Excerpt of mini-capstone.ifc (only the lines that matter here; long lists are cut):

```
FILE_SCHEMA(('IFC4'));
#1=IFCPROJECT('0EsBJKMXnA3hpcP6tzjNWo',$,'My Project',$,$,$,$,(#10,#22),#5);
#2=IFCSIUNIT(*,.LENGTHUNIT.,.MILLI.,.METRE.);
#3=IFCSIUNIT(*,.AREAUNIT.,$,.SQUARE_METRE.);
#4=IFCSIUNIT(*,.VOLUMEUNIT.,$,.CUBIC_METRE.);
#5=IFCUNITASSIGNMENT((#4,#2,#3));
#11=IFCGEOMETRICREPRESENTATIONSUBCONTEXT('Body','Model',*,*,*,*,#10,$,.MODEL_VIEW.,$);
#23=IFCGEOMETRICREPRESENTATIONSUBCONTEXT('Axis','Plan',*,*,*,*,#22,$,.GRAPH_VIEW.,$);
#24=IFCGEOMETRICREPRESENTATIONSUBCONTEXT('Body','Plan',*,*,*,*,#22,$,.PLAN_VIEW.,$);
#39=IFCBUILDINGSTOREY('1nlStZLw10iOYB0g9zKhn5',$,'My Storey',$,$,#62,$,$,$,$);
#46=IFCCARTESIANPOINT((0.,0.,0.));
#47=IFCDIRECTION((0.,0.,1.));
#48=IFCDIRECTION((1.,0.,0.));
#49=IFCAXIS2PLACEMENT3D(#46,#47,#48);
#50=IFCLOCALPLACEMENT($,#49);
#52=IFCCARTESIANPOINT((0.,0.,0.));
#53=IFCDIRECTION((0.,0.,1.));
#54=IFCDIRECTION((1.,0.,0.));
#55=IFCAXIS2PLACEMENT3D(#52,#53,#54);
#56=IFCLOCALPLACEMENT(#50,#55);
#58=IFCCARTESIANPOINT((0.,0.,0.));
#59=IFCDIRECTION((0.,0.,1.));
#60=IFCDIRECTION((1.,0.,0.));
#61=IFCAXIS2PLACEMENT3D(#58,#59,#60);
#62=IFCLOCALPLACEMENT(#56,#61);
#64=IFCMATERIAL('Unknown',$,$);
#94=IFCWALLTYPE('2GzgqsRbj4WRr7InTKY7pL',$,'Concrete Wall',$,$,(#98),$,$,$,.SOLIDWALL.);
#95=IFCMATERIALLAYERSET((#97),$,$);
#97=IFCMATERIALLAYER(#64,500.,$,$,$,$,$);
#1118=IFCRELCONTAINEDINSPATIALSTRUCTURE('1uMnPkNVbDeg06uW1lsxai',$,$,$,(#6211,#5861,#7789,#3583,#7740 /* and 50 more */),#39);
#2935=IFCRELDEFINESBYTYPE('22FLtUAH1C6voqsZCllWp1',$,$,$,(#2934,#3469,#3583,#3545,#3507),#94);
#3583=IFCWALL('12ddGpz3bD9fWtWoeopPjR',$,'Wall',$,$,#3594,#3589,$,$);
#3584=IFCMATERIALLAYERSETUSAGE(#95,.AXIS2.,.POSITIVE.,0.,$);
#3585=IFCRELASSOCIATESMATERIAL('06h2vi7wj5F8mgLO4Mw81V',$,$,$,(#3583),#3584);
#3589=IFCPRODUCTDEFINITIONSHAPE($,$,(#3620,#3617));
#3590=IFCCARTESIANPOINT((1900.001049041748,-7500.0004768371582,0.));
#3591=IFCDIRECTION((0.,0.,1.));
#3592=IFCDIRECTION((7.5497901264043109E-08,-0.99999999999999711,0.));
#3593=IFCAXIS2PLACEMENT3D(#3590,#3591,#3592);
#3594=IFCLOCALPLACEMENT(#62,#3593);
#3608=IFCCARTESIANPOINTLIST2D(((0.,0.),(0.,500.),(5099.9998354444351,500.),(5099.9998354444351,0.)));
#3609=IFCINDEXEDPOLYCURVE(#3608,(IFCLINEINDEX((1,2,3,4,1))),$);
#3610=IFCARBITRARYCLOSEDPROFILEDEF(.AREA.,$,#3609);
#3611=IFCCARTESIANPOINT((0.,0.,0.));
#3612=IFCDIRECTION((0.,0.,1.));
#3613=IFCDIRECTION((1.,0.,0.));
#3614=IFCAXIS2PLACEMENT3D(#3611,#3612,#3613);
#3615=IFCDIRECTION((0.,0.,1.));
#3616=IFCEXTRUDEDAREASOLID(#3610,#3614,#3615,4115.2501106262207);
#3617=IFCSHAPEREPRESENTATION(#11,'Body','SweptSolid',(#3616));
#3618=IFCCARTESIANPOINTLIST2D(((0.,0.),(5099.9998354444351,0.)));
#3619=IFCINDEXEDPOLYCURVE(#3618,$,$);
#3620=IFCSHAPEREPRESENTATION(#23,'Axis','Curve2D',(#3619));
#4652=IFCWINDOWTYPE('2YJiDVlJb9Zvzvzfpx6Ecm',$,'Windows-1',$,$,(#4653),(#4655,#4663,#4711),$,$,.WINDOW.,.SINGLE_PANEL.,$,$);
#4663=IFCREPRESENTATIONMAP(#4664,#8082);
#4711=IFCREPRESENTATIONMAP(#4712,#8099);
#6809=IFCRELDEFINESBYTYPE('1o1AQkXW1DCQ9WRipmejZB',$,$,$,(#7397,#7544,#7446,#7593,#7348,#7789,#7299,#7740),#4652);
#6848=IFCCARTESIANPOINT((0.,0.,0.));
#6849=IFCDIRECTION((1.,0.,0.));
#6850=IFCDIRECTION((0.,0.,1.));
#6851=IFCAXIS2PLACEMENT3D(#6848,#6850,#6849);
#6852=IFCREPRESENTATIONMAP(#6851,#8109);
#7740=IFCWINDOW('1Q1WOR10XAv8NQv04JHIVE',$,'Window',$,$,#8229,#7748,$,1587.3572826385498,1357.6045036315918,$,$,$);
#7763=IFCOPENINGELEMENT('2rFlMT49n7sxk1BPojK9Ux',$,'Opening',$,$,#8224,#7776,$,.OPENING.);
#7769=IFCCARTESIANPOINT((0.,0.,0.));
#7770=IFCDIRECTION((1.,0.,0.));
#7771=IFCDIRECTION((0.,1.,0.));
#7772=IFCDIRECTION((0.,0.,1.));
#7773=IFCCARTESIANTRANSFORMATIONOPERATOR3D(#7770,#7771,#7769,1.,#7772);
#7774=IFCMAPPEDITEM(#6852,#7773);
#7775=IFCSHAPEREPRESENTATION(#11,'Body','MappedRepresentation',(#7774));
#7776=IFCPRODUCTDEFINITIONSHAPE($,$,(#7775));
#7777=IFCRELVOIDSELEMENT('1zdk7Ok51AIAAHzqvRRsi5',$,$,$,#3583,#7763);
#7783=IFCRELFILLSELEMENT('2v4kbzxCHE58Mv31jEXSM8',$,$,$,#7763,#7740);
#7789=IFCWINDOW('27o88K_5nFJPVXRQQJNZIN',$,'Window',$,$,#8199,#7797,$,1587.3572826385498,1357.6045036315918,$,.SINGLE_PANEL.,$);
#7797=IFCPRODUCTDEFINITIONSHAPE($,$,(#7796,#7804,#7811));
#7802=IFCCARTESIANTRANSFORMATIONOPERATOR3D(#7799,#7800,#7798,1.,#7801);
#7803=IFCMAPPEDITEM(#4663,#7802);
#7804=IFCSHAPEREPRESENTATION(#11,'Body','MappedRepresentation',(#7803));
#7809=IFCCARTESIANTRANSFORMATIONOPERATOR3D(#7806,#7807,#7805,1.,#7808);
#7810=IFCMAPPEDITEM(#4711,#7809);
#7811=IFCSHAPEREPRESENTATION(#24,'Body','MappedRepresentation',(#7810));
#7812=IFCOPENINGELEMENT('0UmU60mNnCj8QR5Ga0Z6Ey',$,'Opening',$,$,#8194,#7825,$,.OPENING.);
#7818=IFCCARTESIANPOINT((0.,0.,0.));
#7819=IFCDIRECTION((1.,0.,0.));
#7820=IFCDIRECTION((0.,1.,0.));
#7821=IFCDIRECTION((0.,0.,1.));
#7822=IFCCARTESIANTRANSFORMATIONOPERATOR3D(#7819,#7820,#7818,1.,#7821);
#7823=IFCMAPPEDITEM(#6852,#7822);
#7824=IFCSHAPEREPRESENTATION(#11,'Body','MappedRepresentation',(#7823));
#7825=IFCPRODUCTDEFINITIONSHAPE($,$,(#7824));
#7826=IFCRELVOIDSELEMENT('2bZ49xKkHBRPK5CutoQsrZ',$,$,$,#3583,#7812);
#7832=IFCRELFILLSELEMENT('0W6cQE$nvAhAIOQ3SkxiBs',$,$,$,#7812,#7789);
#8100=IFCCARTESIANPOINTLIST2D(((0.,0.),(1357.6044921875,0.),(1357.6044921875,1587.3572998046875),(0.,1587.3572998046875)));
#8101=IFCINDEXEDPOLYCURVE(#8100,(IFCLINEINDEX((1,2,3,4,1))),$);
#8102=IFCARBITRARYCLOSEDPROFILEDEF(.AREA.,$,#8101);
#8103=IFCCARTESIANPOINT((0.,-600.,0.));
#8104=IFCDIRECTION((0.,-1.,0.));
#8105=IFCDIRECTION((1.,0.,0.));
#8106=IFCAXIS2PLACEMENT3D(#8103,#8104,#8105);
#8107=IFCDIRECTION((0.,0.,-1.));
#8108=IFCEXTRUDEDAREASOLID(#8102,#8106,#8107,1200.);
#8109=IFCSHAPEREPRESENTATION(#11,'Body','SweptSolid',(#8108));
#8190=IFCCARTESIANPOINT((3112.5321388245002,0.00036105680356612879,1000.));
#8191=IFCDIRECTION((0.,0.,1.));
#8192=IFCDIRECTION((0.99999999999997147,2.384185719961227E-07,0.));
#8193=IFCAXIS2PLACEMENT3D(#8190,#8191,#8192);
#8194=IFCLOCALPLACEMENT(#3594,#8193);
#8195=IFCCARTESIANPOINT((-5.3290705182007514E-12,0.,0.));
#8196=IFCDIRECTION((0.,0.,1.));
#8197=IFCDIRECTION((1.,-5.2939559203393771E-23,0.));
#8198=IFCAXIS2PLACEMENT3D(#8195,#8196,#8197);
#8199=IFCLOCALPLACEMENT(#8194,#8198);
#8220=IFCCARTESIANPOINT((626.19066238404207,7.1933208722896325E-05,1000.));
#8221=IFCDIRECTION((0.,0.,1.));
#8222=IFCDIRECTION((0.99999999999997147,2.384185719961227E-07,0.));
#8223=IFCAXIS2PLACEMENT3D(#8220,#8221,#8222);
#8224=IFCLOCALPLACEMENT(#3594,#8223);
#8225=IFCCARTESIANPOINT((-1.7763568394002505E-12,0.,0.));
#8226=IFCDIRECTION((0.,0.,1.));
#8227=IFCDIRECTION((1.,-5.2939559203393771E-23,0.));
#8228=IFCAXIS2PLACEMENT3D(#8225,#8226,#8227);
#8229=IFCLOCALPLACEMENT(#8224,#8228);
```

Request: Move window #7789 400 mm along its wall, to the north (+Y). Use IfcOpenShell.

```python
import ifcopenshell
import ifcopenshell.api.geometry
import ifcopenshell.util.placement
import ifcopenshell.util.unit

model = ifcopenshell.open("mini-capstone.ifc")
unit_scale = ifcopenshell.util.unit.calculate_unit_scale(model)

window = model.by_id(7789)
opening = window.FillsVoids[0].RelatingOpeningElement
wall = opening.VoidsElements[0].RelatingBuildingElement

wall_matrix = ifcopenshell.util.placement.get_local_placement(wall.ObjectPlacement)
shift = wall_matrix[:3, 0] * -0.4 / unit_scale
before = ifcopenshell.util.placement.get_local_placement(window.ObjectPlacement)[:3, 3].copy()

# The window is placed relative to its opening, so it follows when the opening moves.
matrix = ifcopenshell.util.placement.get_local_placement(opening.ObjectPlacement)
matrix[:3, 3] += shift
ifcopenshell.api.geometry.edit_object_placement(
    model, product=opening, matrix=matrix, is_si=False, should_transform_children=True
)

after = ifcopenshell.util.placement.get_local_placement(window.ObjectPlacement)[:3, 3]
print("window moved by", (after - before).round(3) + 0.0)

model.write("mini-capstone_v2.ifc")
```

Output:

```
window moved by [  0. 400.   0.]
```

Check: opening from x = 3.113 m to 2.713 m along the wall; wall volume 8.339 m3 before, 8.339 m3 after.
